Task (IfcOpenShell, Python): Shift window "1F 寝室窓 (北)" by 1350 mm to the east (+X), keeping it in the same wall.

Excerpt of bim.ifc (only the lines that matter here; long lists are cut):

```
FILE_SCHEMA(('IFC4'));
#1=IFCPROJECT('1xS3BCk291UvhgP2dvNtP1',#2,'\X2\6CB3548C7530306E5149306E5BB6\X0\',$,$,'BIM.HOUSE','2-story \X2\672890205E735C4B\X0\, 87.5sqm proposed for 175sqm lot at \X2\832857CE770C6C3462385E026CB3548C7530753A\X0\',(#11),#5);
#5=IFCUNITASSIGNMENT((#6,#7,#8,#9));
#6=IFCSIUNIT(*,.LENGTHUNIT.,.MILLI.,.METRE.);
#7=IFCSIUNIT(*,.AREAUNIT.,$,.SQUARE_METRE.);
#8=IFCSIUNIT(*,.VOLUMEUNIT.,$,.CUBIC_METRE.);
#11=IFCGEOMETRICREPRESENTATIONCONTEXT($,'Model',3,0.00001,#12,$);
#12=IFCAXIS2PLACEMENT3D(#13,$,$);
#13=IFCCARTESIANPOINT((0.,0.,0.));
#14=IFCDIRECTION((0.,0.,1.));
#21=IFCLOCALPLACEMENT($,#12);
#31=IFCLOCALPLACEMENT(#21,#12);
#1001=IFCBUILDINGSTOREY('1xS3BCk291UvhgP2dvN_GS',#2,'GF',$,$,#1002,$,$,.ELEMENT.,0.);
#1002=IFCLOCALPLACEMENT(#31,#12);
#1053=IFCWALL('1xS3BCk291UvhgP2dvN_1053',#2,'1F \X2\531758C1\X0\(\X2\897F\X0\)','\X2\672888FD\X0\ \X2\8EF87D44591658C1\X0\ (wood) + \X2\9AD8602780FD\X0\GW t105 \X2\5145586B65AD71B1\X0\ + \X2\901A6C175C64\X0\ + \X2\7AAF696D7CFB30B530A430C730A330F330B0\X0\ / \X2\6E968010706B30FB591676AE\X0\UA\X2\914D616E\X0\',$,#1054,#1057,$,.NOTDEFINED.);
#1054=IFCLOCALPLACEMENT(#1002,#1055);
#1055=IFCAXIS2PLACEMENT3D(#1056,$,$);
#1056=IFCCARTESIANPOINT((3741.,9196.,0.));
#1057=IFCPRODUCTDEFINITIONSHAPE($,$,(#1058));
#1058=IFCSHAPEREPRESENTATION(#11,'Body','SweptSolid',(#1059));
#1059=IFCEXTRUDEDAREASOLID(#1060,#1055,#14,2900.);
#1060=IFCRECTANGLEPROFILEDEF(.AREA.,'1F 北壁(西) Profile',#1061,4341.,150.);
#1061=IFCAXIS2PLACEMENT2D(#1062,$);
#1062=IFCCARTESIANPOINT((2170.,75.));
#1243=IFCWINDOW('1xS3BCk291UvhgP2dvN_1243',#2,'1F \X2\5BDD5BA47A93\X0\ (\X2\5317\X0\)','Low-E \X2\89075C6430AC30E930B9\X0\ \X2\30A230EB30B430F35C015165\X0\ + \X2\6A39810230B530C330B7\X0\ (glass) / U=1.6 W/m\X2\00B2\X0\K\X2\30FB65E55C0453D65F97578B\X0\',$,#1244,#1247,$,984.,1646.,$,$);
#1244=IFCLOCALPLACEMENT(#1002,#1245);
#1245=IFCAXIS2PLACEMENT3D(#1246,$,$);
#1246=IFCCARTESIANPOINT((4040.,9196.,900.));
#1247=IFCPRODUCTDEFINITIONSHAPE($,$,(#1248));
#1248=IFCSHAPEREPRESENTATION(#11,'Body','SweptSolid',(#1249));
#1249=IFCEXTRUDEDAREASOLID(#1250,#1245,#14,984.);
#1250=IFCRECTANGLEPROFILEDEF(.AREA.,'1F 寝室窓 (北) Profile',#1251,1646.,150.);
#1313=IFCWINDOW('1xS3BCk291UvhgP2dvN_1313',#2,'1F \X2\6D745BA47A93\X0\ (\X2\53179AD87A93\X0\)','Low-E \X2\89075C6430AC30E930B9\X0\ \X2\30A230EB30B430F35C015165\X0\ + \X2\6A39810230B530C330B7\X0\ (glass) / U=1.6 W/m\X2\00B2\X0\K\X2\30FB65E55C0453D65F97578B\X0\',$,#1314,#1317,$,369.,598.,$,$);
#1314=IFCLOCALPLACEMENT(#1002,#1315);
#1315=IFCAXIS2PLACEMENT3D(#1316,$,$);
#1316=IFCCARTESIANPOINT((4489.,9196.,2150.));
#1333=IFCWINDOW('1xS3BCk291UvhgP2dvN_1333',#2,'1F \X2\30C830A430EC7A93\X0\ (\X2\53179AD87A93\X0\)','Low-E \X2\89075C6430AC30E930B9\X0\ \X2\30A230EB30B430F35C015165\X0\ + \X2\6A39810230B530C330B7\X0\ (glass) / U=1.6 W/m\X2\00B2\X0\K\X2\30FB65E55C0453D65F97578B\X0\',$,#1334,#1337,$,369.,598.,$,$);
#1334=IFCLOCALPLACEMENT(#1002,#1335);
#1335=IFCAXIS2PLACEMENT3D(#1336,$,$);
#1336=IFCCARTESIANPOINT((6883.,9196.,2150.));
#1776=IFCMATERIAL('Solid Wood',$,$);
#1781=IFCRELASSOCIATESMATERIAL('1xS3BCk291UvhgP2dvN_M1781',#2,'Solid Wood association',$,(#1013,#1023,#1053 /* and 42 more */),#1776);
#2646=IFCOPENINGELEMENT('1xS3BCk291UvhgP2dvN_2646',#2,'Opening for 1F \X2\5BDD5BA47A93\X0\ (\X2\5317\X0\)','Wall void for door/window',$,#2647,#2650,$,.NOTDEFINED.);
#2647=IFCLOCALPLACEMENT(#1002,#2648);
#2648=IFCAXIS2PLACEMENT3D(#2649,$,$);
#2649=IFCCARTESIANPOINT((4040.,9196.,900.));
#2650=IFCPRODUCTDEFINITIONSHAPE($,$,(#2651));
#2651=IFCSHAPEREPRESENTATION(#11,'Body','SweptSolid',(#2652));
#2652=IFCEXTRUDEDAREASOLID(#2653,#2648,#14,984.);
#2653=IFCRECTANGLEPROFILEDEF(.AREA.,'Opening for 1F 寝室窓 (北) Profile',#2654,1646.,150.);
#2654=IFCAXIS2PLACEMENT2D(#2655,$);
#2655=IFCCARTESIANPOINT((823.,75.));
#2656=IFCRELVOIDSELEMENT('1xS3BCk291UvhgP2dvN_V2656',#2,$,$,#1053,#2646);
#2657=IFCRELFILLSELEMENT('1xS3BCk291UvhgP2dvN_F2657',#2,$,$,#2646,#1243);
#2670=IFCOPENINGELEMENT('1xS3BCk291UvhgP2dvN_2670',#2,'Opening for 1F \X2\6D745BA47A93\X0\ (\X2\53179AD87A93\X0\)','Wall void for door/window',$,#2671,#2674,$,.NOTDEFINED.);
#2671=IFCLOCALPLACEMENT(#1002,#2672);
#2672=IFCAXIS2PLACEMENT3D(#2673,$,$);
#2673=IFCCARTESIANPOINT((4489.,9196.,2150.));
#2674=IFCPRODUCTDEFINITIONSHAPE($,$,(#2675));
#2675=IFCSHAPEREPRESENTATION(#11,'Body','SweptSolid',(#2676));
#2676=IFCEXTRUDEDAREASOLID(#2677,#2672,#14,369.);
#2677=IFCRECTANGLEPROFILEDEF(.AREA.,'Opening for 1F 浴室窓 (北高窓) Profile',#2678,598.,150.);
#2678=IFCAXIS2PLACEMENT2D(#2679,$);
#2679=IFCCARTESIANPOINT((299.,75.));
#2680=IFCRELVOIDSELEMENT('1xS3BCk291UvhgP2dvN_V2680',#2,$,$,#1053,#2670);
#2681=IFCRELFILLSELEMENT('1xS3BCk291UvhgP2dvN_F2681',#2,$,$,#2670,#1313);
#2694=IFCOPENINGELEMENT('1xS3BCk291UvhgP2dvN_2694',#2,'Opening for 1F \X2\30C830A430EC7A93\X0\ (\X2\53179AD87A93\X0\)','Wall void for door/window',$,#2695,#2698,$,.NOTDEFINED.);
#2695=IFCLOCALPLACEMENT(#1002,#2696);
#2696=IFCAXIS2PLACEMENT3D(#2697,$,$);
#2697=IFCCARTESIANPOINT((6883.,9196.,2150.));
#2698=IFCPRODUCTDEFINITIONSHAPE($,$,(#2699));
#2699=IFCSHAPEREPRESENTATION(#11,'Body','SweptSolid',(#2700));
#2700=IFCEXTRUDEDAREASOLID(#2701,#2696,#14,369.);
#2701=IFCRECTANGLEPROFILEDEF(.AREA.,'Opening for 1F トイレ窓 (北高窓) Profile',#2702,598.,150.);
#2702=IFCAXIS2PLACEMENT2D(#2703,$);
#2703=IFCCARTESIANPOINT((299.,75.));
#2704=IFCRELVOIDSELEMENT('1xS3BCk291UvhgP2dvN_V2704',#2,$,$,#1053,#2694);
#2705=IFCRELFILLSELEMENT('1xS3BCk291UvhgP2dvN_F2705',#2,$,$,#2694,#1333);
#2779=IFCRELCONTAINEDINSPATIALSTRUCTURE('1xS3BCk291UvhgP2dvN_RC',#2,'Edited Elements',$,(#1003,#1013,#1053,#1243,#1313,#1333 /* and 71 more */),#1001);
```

```python
import ifcopenshell
import ifcopenshell.api.geometry
import ifcopenshell.util.placement
import ifcopenshell.util.unit

model = ifcopenshell.open("bim.ifc")
unit_scale = ifcopenshell.util.unit.calculate_unit_scale(model)

window = model.by_id(1243)
opening = window.FillsVoids[0].RelatingOpeningElement
wall = opening.VoidsElements[0].RelatingBuildingElement

wall_matrix = ifcopenshell.util.placement.get_local_placement(wall.ObjectPlacement)
shift = wall_matrix[:3, 0] * 1.35 / unit_scale
before = ifcopenshell.util.placement.get_local_placement(window.ObjectPlacement)[:3, 3].copy()

# The window is not placed relative to its opening, so move both.
for product in (opening, window):
    matrix = ifcopenshell.util.placement.get_local_placement(product.ObjectPlacement)
    matrix[:3, 3] += shift
    ifcopenshell.api.geometry.edit_object_placement(model, product=product, matrix=matrix, is_si=False)

after = ifcopenshell.util.placement.get_local_placement(window.ObjectPlacement)[:3, 3]
print("window moved by", (after - before).round(3) + 0.0)

model.write("bim-out.ifc")
```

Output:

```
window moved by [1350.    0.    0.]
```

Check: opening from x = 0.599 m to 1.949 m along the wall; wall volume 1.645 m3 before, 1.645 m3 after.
